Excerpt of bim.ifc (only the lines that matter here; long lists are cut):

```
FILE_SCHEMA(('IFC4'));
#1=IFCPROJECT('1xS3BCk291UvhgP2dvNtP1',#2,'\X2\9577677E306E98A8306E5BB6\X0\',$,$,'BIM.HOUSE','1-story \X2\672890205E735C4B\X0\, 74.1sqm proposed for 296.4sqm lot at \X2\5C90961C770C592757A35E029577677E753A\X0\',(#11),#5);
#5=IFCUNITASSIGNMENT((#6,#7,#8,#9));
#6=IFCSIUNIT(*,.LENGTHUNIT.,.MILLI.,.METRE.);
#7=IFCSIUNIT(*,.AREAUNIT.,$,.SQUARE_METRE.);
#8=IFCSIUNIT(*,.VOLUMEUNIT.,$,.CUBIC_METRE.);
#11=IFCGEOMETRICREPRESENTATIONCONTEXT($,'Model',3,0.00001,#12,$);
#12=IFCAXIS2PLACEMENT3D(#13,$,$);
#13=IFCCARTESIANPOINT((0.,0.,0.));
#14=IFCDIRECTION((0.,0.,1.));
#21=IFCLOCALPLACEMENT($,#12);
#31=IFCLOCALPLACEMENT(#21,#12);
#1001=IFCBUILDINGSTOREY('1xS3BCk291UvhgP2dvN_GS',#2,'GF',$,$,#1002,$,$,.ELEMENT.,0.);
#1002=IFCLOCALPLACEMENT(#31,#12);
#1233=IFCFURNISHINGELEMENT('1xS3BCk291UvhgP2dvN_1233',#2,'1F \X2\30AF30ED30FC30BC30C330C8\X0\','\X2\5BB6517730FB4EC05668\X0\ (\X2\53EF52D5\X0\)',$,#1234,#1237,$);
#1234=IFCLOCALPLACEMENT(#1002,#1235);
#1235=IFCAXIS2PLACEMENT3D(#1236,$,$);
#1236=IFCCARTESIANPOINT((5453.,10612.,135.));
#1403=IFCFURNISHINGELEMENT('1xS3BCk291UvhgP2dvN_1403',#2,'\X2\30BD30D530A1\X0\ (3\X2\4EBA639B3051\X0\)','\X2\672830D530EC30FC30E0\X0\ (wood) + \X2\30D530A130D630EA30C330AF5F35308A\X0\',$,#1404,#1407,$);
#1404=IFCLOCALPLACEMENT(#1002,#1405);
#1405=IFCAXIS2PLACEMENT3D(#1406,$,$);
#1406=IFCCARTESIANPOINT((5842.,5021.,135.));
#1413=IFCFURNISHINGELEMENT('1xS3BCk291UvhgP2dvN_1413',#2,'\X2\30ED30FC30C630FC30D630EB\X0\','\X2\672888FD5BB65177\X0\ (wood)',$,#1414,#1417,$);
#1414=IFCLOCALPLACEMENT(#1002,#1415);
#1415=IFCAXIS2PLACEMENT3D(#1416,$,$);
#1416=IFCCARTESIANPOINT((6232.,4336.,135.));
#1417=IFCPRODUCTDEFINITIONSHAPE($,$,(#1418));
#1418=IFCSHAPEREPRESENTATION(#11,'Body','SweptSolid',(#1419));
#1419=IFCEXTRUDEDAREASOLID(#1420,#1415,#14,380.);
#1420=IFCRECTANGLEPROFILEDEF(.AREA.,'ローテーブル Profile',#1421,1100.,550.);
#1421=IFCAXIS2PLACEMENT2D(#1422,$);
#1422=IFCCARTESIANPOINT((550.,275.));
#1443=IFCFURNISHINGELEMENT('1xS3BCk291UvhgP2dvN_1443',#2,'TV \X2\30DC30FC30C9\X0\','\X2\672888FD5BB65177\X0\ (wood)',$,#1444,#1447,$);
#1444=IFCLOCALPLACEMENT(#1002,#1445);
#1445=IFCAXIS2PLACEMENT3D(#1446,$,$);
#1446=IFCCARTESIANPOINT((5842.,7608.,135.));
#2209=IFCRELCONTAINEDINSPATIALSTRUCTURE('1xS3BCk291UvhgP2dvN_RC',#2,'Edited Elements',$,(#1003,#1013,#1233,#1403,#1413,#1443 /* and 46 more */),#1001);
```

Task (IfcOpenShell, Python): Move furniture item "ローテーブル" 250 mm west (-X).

```python
import ifcopenshell
import ifcopenshell.api.geometry
import ifcopenshell.util.placement

model = ifcopenshell.open("bim.ifc")

item = model.by_guid("1xS3BCk291UvhgP2dvN_1413")
matrix = ifcopenshell.util.placement.get_local_placement(item.ObjectPlacement)
matrix[0, 3] -= 250.0
ifcopenshell.api.geometry.edit_object_placement(model, product=item, matrix=matrix, is_si=False)

print(ifcopenshell.util.placement.get_local_placement(item.ObjectPlacement).round(3) + 0.0)

model.write("bim_v2.ifc")
```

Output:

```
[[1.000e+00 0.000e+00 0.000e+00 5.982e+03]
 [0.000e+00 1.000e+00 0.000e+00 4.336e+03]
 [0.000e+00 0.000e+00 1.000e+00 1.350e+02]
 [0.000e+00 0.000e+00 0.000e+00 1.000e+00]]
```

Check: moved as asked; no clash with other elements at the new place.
